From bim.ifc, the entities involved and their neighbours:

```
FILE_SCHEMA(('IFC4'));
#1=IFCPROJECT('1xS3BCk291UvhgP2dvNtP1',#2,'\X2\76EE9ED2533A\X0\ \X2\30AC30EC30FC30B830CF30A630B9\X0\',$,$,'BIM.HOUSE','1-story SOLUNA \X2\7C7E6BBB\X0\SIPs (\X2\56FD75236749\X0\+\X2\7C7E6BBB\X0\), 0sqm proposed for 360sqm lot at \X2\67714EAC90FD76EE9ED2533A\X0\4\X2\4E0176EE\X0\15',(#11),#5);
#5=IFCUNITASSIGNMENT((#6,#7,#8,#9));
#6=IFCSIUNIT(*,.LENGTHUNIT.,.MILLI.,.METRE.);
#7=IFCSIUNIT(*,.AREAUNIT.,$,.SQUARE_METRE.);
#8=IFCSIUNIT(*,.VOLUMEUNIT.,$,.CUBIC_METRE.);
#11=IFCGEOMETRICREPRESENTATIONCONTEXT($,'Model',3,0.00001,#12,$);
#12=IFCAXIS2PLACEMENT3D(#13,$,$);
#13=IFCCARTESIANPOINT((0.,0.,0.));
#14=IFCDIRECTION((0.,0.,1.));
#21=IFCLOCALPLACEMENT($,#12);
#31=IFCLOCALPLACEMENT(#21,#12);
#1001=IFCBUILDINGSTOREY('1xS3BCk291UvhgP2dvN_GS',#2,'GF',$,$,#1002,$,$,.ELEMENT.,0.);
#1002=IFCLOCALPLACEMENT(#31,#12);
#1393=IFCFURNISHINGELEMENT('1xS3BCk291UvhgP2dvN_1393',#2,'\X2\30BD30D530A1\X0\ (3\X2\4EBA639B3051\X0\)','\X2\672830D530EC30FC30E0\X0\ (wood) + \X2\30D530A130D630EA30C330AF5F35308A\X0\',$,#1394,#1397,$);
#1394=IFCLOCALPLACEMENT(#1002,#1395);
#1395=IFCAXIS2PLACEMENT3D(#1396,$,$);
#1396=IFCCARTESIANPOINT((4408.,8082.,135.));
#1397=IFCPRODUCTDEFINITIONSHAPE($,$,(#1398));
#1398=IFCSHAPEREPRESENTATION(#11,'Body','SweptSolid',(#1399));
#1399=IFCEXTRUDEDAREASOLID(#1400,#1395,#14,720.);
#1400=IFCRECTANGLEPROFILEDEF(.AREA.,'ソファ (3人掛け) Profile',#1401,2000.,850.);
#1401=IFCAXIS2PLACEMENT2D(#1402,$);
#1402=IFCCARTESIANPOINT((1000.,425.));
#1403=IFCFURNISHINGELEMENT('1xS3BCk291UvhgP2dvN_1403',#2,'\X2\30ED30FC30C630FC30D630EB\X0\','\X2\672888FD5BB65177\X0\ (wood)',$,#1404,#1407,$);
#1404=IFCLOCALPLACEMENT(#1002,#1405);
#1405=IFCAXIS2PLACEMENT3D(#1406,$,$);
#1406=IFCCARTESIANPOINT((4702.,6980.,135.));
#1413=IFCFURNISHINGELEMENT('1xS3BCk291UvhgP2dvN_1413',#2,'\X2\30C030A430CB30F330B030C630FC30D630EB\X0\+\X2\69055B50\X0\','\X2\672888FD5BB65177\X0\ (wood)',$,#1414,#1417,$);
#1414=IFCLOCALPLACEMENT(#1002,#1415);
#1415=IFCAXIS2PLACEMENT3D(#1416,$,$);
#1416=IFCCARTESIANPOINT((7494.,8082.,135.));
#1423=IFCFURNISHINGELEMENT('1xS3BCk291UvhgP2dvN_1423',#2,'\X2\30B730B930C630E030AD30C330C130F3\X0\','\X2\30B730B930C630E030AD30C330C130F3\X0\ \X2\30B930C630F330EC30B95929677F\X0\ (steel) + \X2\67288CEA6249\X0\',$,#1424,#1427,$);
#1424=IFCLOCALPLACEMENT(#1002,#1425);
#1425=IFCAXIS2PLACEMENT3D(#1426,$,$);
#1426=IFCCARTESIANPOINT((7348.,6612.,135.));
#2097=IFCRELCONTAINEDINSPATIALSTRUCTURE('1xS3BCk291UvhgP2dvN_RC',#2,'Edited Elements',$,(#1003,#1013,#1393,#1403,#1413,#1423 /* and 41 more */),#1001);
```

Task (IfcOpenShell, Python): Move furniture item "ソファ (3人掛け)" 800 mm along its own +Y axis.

```python
import ifcopenshell
import ifcopenshell.api.geometry
import ifcopenshell.util.placement
import ifcopenshell.util.unit

model = ifcopenshell.open("bim.ifc")
unit_scale = ifcopenshell.util.unit.calculate_unit_scale(model)

item = model.by_guid("1xS3BCk291UvhgP2dvN_1393")
matrix = ifcopenshell.util.placement.get_local_placement(item.ObjectPlacement)
matrix[:3, 3] += matrix[:3, 1] * 0.8 / unit_scale
ifcopenshell.api.geometry.edit_object_placement(model, product=item, matrix=matrix, is_si=False)

print(ifcopenshell.util.placement.get_local_placement(item.ObjectPlacement).round(3) + 0.0)

model.write("bim_v2.ifc")
```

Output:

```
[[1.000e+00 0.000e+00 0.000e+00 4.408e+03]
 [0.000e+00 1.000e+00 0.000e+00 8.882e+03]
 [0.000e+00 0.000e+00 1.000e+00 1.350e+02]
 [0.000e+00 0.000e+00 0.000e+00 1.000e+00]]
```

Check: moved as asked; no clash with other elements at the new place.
